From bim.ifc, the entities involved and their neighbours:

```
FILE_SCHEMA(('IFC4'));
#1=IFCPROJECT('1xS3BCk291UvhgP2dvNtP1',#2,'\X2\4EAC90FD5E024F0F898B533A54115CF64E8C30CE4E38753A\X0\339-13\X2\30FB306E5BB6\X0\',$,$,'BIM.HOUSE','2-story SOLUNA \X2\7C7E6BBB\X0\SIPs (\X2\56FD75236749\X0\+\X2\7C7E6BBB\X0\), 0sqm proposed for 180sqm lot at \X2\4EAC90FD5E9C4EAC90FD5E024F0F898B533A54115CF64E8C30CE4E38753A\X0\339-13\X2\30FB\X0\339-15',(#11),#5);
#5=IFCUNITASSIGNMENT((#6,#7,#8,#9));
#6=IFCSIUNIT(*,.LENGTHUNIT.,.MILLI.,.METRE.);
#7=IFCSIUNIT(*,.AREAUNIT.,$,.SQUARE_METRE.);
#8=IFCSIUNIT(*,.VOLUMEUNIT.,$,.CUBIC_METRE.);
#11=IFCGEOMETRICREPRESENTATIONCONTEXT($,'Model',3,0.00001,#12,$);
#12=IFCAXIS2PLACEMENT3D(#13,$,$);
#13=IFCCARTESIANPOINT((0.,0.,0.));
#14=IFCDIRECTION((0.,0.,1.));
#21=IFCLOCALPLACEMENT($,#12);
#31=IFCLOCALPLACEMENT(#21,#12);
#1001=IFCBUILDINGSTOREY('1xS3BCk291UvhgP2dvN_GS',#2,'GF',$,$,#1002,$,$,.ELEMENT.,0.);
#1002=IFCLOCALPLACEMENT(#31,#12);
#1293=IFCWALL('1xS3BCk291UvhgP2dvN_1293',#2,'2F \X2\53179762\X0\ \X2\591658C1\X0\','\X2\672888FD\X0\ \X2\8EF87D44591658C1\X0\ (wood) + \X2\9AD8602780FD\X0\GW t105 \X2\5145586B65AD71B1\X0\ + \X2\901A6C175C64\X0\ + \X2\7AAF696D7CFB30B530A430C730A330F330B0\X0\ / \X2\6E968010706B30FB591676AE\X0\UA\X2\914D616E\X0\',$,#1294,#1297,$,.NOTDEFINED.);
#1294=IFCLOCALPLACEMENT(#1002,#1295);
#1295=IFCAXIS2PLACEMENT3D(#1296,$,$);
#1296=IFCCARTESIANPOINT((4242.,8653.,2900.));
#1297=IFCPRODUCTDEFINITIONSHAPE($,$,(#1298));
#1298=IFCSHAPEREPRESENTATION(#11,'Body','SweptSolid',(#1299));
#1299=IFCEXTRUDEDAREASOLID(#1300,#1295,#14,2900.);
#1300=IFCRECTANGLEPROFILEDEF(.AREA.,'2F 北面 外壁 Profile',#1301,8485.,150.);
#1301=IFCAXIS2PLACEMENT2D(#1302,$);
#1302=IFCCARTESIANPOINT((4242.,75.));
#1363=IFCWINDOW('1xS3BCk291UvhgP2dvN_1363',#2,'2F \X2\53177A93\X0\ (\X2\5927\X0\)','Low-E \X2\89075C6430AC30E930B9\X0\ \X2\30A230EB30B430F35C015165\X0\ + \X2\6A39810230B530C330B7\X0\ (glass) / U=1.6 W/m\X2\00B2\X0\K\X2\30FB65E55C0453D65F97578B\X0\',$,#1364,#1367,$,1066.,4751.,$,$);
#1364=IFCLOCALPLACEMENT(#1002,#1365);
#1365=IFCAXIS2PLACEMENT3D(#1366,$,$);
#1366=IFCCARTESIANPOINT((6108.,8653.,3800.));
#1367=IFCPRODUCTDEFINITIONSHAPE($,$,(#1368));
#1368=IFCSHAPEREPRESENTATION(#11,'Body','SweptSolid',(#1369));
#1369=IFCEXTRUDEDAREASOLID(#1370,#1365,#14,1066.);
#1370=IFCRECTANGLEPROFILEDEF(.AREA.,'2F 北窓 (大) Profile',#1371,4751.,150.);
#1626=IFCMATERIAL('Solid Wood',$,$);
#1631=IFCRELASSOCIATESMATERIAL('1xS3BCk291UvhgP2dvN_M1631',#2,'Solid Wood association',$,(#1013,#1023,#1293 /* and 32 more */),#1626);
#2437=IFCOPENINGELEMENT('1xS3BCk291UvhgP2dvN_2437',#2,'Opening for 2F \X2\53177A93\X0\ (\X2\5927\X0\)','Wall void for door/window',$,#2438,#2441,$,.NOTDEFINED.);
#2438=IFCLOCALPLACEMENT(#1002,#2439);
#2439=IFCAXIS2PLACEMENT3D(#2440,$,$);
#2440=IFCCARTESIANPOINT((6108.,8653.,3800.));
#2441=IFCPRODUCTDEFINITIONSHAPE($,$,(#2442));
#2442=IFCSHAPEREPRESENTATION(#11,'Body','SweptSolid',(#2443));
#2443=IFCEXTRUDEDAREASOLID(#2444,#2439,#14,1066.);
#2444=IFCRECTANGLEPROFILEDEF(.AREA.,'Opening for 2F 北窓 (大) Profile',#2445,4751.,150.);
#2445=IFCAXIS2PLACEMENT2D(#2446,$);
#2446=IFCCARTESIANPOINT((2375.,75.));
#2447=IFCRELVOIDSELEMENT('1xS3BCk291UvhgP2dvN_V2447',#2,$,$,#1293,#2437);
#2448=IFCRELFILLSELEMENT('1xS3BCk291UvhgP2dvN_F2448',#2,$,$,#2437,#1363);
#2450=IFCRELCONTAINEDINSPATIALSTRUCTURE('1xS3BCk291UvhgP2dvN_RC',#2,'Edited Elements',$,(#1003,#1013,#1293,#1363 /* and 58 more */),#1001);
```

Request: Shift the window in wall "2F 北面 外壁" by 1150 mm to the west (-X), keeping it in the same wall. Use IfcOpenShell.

```python
import ifcopenshell
import ifcopenshell.api.geometry
import ifcopenshell.util.placement
import ifcopenshell.util.unit

model = ifcopenshell.open("bim.ifc")
unit_scale = ifcopenshell.util.unit.calculate_unit_scale(model)

window = model.by_id(1363)
opening = window.FillsVoids[0].RelatingOpeningElement
wall = opening.VoidsElements[0].RelatingBuildingElement

wall_matrix = ifcopenshell.util.placement.get_local_placement(wall.ObjectPlacement)
shift = wall_matrix[:3, 0] * -1.15 / unit_scale
before = ifcopenshell.util.placement.get_local_placement(window.ObjectPlacement)[:3, 3].copy()

# The window is not placed relative to its opening, so move both.
for product in (opening, window):
    matrix = ifcopenshell.util.placement.get_local_placement(product.ObjectPlacement)
    matrix[:3, 3] += shift
    ifcopenshell.api.geometry.edit_object_placement(model, product=product, matrix=matrix, is_si=False)

after = ifcopenshell.util.placement.get_local_placement(window.ObjectPlacement)[:3, 3]
print("window moved by", (after - before).round(3) + 0.0)

model.write("bim-out.ifc")
```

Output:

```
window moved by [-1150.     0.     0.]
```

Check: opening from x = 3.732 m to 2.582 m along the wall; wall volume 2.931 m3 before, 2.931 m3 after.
